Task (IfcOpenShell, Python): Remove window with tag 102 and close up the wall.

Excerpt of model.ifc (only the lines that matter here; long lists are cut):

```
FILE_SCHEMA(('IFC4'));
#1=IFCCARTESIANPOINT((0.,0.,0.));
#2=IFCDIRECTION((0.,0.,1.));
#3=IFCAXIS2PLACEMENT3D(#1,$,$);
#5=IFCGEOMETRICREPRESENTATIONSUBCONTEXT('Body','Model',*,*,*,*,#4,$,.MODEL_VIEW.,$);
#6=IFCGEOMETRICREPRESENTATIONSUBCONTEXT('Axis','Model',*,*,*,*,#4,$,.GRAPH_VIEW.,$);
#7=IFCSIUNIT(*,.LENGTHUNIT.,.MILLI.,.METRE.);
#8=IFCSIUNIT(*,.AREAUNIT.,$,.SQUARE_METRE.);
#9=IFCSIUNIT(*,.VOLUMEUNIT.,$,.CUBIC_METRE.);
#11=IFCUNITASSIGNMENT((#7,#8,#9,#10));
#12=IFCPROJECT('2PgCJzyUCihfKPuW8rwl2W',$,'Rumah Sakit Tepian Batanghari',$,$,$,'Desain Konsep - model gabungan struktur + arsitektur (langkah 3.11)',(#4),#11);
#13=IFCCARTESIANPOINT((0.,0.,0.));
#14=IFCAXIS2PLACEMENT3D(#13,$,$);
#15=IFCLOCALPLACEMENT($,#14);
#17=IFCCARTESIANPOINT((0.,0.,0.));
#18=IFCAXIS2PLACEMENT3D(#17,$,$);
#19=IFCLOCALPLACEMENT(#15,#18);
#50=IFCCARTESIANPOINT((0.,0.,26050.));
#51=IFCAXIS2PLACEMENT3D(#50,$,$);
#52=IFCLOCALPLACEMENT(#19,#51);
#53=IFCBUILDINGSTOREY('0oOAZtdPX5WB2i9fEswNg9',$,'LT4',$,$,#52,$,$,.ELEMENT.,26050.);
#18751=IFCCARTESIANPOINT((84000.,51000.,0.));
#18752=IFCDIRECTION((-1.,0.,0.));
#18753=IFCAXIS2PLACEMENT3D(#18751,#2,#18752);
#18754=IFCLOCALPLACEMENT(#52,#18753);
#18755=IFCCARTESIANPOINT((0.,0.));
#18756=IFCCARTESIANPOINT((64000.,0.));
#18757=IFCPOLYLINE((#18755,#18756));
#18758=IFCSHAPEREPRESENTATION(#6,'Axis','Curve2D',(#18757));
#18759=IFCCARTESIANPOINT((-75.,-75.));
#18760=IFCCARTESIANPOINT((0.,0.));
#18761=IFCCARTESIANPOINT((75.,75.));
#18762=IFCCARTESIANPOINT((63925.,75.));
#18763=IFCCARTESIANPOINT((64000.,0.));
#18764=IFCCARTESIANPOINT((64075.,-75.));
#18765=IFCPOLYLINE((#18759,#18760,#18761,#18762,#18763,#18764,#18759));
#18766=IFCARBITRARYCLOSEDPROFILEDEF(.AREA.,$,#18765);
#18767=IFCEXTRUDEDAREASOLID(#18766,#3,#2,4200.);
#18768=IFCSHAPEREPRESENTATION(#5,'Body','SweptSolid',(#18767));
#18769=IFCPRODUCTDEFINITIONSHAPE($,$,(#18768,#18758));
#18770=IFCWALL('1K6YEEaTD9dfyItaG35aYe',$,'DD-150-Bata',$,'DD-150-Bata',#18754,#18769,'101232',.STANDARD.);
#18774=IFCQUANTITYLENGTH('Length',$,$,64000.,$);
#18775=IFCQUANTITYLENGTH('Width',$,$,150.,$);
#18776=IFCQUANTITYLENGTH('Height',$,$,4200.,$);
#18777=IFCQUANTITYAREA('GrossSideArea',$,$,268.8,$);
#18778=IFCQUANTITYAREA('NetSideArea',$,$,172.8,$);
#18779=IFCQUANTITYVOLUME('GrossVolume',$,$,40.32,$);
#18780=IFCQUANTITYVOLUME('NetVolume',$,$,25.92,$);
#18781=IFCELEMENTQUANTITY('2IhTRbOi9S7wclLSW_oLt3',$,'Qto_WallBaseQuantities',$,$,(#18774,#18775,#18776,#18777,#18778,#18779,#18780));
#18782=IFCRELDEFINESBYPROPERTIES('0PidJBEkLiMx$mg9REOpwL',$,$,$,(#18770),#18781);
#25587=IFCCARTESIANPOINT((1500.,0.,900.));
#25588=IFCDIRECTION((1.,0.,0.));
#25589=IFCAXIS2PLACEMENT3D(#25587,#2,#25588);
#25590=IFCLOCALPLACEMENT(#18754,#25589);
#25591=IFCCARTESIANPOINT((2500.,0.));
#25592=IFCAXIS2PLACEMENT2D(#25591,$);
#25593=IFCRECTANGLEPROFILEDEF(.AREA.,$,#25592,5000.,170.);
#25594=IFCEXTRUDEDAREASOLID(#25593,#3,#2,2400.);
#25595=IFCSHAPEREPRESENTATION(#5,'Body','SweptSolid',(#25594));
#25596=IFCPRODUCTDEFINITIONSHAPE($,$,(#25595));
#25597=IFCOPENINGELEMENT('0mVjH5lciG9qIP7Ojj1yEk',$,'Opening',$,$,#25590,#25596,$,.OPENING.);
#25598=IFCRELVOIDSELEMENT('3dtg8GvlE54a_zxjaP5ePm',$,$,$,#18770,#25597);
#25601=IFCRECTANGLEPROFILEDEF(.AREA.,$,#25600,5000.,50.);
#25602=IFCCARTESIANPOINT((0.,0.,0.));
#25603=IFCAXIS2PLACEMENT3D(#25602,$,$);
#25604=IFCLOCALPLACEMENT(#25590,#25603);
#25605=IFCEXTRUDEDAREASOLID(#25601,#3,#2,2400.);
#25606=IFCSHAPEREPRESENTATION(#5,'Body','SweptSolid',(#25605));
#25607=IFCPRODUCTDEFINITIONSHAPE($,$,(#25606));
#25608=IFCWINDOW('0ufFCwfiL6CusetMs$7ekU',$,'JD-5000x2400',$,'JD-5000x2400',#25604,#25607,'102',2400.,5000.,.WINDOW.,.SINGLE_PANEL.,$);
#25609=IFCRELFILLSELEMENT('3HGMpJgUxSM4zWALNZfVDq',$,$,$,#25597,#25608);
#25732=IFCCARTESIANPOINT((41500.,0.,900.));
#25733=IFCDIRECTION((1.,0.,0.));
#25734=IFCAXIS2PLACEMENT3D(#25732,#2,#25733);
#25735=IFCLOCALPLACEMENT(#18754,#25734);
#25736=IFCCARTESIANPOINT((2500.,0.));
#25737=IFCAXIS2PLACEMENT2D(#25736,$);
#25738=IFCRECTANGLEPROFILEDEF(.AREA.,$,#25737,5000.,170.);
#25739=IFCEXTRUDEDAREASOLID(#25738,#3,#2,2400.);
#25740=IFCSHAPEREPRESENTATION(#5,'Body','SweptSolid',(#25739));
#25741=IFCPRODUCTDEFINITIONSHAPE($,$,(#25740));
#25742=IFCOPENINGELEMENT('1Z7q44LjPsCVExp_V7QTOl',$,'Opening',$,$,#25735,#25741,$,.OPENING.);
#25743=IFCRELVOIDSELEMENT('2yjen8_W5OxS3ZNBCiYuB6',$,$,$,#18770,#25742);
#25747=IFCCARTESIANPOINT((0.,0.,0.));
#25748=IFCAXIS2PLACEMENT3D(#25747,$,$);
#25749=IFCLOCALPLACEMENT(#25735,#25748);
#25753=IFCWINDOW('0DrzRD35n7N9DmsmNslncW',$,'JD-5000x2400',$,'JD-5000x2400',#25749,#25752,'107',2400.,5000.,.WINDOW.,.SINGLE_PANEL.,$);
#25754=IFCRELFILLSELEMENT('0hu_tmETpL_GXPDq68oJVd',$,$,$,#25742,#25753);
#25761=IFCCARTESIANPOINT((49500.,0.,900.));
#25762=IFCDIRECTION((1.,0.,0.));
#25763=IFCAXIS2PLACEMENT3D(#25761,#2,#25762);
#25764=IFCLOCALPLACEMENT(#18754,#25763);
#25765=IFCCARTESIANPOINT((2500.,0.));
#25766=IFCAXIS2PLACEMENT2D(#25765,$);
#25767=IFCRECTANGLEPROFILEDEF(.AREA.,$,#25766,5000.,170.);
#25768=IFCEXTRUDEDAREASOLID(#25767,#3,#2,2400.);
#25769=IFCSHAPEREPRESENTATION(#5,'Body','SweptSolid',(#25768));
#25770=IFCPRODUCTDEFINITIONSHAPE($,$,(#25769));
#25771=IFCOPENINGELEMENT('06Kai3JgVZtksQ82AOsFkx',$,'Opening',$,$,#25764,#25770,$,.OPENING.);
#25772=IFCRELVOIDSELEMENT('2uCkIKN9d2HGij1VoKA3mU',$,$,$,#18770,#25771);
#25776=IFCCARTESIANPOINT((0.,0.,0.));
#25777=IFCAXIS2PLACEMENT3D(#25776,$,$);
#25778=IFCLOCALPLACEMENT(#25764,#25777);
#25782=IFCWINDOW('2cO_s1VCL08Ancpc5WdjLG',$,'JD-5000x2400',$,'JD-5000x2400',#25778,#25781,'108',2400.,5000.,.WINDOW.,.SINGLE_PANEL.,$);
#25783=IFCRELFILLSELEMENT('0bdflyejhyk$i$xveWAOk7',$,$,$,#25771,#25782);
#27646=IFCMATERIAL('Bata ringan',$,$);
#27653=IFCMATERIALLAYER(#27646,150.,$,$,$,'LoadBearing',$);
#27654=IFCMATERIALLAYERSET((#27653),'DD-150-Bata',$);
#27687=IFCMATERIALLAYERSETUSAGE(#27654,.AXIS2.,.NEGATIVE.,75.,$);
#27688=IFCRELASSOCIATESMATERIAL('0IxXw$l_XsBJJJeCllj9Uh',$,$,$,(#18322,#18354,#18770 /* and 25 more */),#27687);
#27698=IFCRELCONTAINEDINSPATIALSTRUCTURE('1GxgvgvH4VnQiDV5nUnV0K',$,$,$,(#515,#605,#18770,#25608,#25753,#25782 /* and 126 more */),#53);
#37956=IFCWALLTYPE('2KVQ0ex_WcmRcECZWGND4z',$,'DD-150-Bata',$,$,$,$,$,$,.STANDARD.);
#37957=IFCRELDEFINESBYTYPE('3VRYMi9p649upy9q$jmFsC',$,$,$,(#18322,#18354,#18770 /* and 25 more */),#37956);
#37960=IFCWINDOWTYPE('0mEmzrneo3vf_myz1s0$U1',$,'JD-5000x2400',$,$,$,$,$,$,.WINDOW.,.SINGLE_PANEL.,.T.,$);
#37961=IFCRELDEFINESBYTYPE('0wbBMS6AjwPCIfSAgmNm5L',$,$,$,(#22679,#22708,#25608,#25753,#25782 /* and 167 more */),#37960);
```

```python
import ifcopenshell
import ifcopenshell.api.feature
import ifcopenshell.api.pset
import ifcopenshell.api.root
import ifcopenshell.geom
import ifcopenshell.util.element
import ifcopenshell.util.shape
import ifcopenshell.util.unit

model = ifcopenshell.open("model.ifc")
area_scale = ifcopenshell.util.unit.calculate_unit_scale(model, "AREAUNIT")
volume_scale = ifcopenshell.util.unit.calculate_unit_scale(model, "VOLUMEUNIT")
settings = ifcopenshell.geom.settings()


def volume(element):
    """Net volume in cubic metres, openings subtracted."""
    shape = ifcopenshell.geom.create_shape(settings, element)
    return ifcopenshell.util.shape.get_volume(shape.geometry)


window = model.by_guid("0ufFCwfiL6CusetMs$7ekU")
opening = window.FillsVoids[0].RelatingOpeningElement
wall = opening.VoidsElements[0].RelatingBuildingElement
before = volume(wall)

ifcopenshell.api.root.remove_product(model, product=window)
ifcopenshell.api.feature.remove_feature(model, feature=opening)

after = volume(wall)
thickness = 0.15  # wall thickness in metres

# Update the wall's stored quantities.
qto = model.by_id(ifcopenshell.util.element.get_pset(wall, "Qto_WallBaseQuantities", should_inherit=False)["id"])
ifcopenshell.api.pset.edit_qto(model, qto=qto, properties={
    "NetSideArea": after / thickness / area_scale,
    "NetVolume": after / volume_scale,
})

print(f"wall volume {before:.3f} -> {after:.3f} m3")

model.write("model_updated.ifc")
```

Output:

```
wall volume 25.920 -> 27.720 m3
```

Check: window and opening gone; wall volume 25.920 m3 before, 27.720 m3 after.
